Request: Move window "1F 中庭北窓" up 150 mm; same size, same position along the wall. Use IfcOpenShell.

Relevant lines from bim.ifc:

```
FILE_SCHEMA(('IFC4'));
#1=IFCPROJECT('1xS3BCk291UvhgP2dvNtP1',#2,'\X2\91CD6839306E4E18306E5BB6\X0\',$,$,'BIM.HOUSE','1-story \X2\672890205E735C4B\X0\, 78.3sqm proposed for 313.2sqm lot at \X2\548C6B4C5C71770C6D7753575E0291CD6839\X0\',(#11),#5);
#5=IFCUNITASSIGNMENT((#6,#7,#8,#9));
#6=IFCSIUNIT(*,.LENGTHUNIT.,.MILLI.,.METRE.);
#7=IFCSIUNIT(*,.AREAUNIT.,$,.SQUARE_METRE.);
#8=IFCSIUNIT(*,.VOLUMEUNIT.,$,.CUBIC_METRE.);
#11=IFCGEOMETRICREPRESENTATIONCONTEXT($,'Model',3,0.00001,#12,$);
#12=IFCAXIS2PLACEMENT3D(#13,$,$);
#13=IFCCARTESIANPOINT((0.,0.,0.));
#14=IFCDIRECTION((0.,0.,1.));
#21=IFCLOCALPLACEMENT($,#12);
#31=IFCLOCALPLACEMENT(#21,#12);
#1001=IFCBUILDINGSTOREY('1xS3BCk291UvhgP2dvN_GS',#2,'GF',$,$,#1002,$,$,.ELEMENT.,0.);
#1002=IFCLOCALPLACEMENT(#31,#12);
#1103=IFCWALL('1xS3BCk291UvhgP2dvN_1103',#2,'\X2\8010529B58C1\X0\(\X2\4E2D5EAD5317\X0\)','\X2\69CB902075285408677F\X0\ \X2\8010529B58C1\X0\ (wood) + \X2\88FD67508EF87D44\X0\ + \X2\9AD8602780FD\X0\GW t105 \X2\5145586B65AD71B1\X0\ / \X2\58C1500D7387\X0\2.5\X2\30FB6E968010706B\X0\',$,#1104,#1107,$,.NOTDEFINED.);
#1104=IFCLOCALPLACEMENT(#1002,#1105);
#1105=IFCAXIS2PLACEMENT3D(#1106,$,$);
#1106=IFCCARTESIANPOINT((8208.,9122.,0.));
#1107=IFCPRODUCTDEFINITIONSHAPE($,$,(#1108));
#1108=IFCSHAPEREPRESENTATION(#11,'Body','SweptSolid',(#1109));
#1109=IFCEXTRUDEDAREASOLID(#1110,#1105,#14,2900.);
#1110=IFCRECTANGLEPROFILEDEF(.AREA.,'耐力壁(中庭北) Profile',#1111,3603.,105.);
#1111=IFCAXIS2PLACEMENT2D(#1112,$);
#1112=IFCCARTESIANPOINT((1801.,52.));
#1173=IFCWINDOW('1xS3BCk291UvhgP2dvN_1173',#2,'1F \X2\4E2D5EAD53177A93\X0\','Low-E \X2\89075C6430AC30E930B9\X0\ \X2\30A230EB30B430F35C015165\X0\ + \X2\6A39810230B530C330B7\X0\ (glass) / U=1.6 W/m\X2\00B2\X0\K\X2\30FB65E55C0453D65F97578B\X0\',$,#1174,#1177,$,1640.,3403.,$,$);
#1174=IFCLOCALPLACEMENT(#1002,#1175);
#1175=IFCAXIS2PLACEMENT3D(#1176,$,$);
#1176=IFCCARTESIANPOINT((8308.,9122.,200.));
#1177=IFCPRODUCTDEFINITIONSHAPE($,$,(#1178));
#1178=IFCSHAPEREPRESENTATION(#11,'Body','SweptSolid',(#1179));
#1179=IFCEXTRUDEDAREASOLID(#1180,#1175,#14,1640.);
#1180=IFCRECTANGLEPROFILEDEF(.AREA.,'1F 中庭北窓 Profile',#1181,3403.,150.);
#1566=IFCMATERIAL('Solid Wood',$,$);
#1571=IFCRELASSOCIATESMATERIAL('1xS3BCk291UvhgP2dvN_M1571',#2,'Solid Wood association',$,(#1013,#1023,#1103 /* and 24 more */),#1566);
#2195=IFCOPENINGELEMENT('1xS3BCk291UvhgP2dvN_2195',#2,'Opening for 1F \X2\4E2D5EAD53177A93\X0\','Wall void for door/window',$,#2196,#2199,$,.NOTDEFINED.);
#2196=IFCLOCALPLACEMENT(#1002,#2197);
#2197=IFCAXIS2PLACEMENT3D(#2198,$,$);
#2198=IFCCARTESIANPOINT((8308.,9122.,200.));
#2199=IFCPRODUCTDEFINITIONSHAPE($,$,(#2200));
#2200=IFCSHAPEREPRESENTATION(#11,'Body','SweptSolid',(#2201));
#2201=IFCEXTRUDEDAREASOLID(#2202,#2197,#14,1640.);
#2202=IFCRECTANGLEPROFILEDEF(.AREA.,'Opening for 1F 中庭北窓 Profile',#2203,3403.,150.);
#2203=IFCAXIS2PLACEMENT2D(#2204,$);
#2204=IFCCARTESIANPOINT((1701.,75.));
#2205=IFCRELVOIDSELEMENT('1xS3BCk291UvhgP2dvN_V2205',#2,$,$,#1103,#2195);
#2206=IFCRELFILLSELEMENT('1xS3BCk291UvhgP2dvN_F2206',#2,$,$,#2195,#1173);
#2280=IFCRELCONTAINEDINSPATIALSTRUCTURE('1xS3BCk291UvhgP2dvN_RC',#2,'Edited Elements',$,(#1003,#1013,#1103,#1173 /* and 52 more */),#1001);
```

```python
import numpy as np
import ifcopenshell
import ifcopenshell.api.geometry
import ifcopenshell.util.placement
import ifcopenshell.util.unit

model = ifcopenshell.open("bim.ifc")
unit_scale = ifcopenshell.util.unit.calculate_unit_scale(model)

window = model.by_guid("1xS3BCk291UvhgP2dvN_1173")
opening = window.FillsVoids[0].RelatingOpeningElement
dz = 150.0

shift = np.array([0.0, 0.0, dz])
# The window is not placed relative to its opening, so move both.
for product in (opening, window):
    matrix = ifcopenshell.util.placement.get_local_placement(product.ObjectPlacement)
    matrix[:3, 3] += shift
    ifcopenshell.api.geometry.edit_object_placement(model, product=product, matrix=matrix, is_si=False)

print(f"moved by {dz * unit_scale:+.3f} m")

model.write("bim_rev.ifc")
```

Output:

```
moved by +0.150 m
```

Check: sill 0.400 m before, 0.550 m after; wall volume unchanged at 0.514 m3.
